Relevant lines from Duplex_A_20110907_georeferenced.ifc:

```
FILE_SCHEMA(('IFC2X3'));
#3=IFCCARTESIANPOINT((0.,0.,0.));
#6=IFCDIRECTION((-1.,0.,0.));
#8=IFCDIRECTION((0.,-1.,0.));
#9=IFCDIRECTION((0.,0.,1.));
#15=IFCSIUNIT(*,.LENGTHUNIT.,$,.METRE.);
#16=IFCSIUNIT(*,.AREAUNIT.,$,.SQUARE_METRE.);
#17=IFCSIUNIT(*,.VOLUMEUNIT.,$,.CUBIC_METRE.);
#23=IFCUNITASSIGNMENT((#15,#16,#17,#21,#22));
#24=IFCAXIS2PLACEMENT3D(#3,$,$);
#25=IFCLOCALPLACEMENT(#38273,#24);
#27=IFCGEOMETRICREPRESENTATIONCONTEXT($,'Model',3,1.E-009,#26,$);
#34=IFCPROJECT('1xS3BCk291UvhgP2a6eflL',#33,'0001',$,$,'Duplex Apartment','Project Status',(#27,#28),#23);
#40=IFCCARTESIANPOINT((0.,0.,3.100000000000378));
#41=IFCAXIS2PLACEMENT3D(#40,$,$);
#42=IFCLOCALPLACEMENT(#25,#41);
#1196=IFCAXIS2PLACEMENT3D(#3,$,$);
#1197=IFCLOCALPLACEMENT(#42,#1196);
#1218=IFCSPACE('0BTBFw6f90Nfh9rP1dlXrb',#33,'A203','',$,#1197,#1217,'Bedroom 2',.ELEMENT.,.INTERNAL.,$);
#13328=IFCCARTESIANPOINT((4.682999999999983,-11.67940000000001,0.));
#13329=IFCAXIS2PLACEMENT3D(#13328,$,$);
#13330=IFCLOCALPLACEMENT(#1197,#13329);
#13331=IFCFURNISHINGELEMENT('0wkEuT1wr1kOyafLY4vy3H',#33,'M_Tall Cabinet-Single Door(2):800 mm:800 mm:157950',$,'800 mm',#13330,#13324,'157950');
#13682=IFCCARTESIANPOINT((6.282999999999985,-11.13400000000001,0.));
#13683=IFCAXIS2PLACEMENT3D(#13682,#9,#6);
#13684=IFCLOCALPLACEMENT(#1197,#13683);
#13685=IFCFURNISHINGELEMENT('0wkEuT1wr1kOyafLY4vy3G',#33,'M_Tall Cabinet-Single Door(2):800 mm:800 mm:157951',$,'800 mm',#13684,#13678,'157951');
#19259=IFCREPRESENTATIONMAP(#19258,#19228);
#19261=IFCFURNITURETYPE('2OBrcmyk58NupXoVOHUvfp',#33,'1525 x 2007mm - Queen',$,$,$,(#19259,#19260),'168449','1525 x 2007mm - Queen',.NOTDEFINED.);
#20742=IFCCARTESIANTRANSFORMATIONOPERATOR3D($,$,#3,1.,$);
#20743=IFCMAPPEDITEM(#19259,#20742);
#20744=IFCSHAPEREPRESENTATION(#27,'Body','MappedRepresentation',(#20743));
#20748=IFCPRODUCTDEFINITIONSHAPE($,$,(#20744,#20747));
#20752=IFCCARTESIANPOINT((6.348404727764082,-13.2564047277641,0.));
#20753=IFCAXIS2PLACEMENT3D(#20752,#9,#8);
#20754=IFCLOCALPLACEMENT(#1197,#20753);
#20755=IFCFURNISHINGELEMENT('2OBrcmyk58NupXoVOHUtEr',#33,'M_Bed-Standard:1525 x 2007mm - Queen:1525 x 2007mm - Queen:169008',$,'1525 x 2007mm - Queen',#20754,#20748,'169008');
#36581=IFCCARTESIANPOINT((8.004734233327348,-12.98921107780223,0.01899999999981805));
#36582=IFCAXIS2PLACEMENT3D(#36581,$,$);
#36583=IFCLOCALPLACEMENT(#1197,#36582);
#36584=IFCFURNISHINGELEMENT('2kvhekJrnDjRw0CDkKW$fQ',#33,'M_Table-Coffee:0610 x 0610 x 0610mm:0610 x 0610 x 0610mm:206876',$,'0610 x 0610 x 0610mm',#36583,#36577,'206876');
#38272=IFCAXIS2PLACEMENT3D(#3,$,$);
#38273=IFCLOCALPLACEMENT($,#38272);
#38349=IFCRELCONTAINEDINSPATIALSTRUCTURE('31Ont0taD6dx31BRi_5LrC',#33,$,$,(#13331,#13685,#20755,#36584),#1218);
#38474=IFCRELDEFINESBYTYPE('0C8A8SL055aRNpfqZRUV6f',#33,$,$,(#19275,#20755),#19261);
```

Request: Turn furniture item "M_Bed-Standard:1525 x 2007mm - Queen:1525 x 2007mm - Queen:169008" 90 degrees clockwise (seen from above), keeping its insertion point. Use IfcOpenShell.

```python
import ifcopenshell
import ifcopenshell.api.geometry
import ifcopenshell.util.placement

model = ifcopenshell.open("Duplex_A_20110907_georeferenced.ifc")

item = model.by_guid("2OBrcmyk58NupXoVOHUtEr")
matrix = ifcopenshell.util.placement.get_local_placement(item.ObjectPlacement)
matrix = matrix @ ifcopenshell.util.placement.rotation(-90, "Z")
ifcopenshell.api.geometry.edit_object_placement(model, product=item, matrix=matrix, is_si=False)

print(ifcopenshell.util.placement.get_local_placement(item.ObjectPlacement).round(3) + 0.0)

model.write("Duplex_A_20110907_georeferenced_edited.ifc")
```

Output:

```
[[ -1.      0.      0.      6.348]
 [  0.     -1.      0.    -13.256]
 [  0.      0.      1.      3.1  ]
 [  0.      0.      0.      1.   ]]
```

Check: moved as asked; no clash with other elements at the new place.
